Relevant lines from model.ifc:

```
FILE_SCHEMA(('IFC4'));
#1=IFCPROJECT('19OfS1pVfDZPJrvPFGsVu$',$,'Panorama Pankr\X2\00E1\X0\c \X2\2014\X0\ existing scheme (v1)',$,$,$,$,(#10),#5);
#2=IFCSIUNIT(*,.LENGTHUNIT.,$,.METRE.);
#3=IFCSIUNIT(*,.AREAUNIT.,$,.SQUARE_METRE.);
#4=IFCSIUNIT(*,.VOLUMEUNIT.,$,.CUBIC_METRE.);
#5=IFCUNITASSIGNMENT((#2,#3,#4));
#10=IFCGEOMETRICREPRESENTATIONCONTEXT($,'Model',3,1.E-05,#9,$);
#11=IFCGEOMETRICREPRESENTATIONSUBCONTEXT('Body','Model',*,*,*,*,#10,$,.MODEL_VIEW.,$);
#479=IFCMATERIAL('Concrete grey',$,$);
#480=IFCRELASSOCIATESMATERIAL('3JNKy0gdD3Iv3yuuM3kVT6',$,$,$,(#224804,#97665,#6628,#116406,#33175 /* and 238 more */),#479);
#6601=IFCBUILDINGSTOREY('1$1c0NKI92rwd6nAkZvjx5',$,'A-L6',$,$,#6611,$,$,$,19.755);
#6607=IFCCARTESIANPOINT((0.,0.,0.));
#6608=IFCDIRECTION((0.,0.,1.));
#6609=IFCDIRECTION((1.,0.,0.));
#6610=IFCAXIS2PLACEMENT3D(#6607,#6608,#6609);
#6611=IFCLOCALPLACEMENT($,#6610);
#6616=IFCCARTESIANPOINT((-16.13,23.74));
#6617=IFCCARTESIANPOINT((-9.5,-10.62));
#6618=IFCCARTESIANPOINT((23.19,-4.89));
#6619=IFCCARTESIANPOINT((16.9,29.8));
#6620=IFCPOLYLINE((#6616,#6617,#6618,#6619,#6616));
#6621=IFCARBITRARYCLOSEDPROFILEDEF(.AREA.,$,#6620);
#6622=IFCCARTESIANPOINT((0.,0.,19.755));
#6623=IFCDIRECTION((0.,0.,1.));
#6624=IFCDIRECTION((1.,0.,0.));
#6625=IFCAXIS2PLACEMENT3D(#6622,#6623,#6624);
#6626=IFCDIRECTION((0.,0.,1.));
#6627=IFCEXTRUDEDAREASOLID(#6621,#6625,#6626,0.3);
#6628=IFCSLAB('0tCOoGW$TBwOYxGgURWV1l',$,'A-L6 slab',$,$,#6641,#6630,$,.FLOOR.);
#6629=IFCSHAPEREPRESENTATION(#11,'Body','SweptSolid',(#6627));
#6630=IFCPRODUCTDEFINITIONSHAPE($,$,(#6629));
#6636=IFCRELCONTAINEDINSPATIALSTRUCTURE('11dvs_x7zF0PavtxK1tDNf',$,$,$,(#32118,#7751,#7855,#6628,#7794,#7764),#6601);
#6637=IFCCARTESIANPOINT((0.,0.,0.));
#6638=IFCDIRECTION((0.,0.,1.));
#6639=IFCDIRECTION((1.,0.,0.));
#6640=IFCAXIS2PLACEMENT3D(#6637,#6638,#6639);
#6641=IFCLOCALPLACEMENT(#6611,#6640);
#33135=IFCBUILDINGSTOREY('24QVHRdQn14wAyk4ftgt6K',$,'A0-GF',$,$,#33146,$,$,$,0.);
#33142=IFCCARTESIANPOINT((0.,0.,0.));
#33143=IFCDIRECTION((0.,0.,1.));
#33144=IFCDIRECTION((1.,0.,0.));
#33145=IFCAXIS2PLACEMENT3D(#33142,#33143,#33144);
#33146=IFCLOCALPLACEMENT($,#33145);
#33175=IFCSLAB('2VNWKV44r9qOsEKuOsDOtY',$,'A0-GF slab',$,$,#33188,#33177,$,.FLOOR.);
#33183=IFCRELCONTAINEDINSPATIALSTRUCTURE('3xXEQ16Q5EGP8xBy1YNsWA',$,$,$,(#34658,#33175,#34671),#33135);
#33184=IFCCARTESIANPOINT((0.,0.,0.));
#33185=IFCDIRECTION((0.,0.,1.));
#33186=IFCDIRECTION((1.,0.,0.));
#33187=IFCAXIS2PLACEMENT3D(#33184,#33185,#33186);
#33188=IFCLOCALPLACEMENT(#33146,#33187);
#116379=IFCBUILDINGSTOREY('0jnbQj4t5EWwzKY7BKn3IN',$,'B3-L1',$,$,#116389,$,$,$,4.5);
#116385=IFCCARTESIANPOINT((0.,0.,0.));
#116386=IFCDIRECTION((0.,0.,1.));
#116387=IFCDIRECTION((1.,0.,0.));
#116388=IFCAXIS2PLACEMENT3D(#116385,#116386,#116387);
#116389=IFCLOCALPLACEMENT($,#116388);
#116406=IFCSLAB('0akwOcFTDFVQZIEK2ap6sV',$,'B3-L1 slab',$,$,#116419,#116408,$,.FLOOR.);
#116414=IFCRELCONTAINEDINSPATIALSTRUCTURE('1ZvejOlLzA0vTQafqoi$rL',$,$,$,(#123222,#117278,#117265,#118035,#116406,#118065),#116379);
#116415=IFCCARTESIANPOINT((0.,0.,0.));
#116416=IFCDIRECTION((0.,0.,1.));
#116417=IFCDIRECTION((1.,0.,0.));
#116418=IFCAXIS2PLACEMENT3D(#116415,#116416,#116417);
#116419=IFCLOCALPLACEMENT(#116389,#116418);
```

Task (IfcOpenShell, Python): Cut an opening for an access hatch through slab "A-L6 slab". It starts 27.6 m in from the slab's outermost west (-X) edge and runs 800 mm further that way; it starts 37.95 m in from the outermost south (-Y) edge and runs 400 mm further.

```python
import numpy as np
import ifcopenshell
import ifcopenshell.api.feature
import ifcopenshell.api.geometry
import ifcopenshell.api.root
import ifcopenshell.geom
import ifcopenshell.util.placement
import ifcopenshell.util.representation
import ifcopenshell.util.shape
import ifcopenshell.util.unit

model = ifcopenshell.open("model.ifc")
unit_scale = ifcopenshell.util.unit.calculate_unit_scale(model)
settings = ifcopenshell.geom.settings()


def volume(element):
    """Net volume in cubic metres, openings subtracted."""
    shape = ifcopenshell.geom.create_shape(settings, element)
    return ifcopenshell.util.shape.get_volume(shape.geometry)


slab = model.by_id(6628)
before = volume(slab)

# Extent in the slab's own axes, in metres. The edges named are its -X and -Y sides.
slab_shape = ifcopenshell.geom.create_shape(settings, slab)
vertices = ifcopenshell.util.shape.get_vertices(slab_shape.geometry)
x_min, y_min, bottom = vertices.min(axis=0)
top = vertices[:, 2].max()

opening = ifcopenshell.api.root.create_entity(model, ifc_class="IfcOpeningElement", name="Access hatch opening", predefined_type="OPENING")
context = ifcopenshell.util.representation.get_context(model, "Model", "Body", "MODEL_VIEW")
width, depth = 0.8, 0.4
outline = [(0.0, 0.0), (width, 0.0), (width, depth), (0.0, depth), (0.0, 0.0)]
# Overshoot both faces by 50 mm so the cut is clean.
shape = ifcopenshell.api.geometry.add_slab_representation(
    model, context=context, depth=top - bottom + 0.1, polyline=outline
)
ifcopenshell.api.geometry.assign_representation(model, product=opening, representation=shape)

matrix = ifcopenshell.util.placement.get_local_placement(slab.ObjectPlacement)
matrix[:, 3] = matrix @ np.append(np.array([x_min + 27.6, y_min + 37.95, bottom - 0.05]) / unit_scale, 1.0)
ifcopenshell.api.geometry.edit_object_placement(model, product=opening, matrix=matrix, is_si=False)
ifcopenshell.api.feature.add_feature(model, feature=opening, element=slab)

after = volume(slab)

print(f"slab volume {before:.3f} -> {after:.3f} m3")

model.write("model_v2.ifc")
```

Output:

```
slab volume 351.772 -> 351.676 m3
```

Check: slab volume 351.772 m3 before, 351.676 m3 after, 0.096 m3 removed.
